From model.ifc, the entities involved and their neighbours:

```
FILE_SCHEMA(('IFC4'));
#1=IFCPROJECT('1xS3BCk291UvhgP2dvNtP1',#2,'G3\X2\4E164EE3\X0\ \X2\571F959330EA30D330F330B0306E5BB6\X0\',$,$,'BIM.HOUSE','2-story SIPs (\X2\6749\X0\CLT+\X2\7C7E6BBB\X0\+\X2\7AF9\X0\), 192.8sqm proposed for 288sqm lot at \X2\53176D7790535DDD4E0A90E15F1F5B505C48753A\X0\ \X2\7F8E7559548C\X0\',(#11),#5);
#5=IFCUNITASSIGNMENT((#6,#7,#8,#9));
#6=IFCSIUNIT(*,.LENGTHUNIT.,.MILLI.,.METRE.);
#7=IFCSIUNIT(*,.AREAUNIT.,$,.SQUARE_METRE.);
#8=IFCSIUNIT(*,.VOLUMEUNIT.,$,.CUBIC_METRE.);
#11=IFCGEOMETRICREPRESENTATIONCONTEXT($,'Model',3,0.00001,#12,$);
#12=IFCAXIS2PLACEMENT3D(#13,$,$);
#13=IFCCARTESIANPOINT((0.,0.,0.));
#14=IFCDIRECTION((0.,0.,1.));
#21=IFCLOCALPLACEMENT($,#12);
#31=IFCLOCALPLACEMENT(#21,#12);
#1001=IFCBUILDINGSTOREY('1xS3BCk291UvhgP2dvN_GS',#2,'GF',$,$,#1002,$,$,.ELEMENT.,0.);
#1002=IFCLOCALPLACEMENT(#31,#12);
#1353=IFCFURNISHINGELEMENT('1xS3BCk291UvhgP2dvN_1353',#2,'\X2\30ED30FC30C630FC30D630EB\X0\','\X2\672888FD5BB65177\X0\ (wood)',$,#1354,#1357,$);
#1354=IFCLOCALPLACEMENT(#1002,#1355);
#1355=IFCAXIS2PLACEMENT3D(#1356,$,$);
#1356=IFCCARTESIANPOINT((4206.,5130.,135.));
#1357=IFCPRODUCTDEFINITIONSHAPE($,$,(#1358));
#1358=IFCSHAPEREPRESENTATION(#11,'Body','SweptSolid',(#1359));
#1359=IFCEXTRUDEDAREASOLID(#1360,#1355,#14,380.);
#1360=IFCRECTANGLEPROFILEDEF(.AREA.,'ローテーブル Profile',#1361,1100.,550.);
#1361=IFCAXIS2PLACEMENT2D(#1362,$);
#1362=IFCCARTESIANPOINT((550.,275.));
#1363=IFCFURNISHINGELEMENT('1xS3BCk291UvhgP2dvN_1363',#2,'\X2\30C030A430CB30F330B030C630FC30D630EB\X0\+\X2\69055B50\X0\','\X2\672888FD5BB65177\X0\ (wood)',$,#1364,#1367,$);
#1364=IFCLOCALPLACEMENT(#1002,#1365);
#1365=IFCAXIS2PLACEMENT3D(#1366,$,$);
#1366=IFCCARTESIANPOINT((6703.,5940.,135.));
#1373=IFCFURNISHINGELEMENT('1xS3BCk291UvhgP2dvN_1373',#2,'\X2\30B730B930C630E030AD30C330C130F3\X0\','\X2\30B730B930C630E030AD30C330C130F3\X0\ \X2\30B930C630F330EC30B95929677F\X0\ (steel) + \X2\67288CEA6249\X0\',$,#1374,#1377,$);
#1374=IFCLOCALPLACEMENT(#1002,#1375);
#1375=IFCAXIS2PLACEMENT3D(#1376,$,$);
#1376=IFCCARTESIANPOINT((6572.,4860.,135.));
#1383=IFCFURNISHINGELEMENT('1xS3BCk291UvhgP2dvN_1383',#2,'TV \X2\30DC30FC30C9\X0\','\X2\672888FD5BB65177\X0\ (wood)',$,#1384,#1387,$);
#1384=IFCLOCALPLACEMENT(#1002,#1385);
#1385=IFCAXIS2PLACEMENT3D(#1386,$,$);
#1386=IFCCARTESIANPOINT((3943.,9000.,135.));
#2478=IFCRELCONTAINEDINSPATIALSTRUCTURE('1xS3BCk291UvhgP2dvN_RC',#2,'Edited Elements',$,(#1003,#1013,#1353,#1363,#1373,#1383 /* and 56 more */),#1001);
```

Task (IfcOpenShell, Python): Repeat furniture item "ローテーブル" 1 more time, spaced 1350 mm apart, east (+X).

```python
import numpy as np
import ifcopenshell
import ifcopenshell.api.geometry
import ifcopenshell.api.root
import ifcopenshell.util.element
import ifcopenshell.util.placement
import ifcopenshell.util.unit

model = ifcopenshell.open("model.ifc")
unit_scale = ifcopenshell.util.unit.calculate_unit_scale(model)


def reuse_history(source, copy):
    """copy_class also copies each property set's owner history, people and application; keep the originals."""
    for rel in copy.IsDefinedBy:
        if rel.is_a("IfcRelDefinesByProperties") and (history := rel.RelatingPropertyDefinition.OwnerHistory):
            rel.RelatingPropertyDefinition.OwnerHistory = source.OwnerHistory
            ifcopenshell.util.element.remove_deep2(model, history)


source = model.by_guid("1xS3BCk291UvhgP2dvN_1353")
base = ifcopenshell.util.placement.get_local_placement(source.ObjectPlacement)
step = np.array([1.0, 0.0, 0.0]) * 1.35 / unit_scale

for i in range(1, 2):
    copy = ifcopenshell.api.root.copy_class(model, product=source)
    copy.Representation = ifcopenshell.util.element.copy_deep(
        model, source.Representation, exclude=["IfcGeometricRepresentationContext", "IfcRepresentationMap"]
    )
    reuse_history(source, copy)
    matrix = base.copy()
    matrix[:3, 3] += i * step
    print("added at", matrix[:3, 3].round(3) + 0.0)
    ifcopenshell.api.geometry.edit_object_placement(model, product=copy, matrix=matrix, is_si=False)

model.write("model_updated.ifc")
```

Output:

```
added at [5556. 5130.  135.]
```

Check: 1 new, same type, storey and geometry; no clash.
